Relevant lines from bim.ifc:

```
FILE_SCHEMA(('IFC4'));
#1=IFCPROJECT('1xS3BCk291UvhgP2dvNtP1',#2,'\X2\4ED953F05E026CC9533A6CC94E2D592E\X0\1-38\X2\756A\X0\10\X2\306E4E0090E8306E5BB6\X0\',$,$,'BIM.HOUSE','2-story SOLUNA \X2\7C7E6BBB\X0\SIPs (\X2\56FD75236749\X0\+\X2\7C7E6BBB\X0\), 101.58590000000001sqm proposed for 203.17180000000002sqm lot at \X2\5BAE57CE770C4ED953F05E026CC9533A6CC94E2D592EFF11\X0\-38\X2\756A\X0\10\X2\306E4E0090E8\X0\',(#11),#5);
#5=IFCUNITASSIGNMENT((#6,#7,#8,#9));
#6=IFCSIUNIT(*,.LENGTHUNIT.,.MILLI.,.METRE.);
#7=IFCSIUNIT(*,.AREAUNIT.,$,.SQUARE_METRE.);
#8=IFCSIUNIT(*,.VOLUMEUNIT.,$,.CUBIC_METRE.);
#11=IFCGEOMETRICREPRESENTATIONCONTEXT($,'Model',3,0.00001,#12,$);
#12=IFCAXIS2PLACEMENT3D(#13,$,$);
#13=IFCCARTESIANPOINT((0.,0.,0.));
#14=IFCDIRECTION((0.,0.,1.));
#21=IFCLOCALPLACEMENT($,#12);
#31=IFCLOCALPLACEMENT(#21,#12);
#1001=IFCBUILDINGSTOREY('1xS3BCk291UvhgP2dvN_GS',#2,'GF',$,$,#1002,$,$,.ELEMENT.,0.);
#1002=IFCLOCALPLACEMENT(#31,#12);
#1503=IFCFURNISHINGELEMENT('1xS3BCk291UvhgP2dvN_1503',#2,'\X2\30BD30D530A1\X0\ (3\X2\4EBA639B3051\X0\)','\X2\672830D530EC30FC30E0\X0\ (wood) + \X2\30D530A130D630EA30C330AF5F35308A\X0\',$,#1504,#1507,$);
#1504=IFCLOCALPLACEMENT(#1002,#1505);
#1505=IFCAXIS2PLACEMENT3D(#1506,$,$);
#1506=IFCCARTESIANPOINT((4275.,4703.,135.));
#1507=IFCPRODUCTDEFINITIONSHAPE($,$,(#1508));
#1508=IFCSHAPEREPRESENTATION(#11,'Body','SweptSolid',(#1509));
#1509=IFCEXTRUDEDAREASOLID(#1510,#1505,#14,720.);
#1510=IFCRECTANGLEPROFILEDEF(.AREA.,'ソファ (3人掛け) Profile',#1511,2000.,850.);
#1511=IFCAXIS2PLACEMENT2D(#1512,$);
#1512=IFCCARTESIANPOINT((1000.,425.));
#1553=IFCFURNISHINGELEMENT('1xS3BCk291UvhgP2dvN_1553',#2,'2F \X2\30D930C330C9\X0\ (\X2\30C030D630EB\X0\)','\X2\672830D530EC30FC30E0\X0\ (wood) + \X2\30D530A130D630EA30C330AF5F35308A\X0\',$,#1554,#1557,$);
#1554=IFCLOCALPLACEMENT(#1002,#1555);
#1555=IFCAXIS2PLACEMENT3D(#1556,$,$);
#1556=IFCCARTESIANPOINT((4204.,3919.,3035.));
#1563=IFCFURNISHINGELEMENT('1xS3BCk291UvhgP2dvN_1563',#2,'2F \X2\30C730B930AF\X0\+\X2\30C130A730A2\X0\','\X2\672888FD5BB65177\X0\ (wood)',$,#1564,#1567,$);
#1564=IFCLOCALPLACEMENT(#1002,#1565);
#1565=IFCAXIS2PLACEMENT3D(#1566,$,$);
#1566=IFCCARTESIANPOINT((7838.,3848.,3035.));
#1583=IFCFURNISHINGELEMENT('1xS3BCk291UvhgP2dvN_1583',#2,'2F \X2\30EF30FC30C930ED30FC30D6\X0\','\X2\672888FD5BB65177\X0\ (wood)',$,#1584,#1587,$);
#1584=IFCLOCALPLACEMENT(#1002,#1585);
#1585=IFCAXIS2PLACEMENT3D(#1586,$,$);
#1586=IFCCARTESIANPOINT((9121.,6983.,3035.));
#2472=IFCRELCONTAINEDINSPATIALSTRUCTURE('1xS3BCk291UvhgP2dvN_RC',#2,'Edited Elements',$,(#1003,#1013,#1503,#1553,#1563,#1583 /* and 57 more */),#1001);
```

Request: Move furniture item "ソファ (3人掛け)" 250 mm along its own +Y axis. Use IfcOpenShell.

```python
import ifcopenshell
import ifcopenshell.api.geometry
import ifcopenshell.util.placement
import ifcopenshell.util.unit

model = ifcopenshell.open("bim.ifc")
unit_scale = ifcopenshell.util.unit.calculate_unit_scale(model)

item = model.by_id(1503)
matrix = ifcopenshell.util.placement.get_local_placement(item.ObjectPlacement)
matrix[:3, 3] += matrix[:3, 1] * 0.25 / unit_scale
ifcopenshell.api.geometry.edit_object_placement(model, product=item, matrix=matrix, is_si=False)

print(ifcopenshell.util.placement.get_local_placement(item.ObjectPlacement).round(3) + 0.0)

model.write("bim-out.ifc")
```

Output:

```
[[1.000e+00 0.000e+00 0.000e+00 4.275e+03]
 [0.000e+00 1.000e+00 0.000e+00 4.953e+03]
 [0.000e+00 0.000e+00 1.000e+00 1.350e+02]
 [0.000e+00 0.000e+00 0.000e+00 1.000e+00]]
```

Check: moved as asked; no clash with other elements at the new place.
